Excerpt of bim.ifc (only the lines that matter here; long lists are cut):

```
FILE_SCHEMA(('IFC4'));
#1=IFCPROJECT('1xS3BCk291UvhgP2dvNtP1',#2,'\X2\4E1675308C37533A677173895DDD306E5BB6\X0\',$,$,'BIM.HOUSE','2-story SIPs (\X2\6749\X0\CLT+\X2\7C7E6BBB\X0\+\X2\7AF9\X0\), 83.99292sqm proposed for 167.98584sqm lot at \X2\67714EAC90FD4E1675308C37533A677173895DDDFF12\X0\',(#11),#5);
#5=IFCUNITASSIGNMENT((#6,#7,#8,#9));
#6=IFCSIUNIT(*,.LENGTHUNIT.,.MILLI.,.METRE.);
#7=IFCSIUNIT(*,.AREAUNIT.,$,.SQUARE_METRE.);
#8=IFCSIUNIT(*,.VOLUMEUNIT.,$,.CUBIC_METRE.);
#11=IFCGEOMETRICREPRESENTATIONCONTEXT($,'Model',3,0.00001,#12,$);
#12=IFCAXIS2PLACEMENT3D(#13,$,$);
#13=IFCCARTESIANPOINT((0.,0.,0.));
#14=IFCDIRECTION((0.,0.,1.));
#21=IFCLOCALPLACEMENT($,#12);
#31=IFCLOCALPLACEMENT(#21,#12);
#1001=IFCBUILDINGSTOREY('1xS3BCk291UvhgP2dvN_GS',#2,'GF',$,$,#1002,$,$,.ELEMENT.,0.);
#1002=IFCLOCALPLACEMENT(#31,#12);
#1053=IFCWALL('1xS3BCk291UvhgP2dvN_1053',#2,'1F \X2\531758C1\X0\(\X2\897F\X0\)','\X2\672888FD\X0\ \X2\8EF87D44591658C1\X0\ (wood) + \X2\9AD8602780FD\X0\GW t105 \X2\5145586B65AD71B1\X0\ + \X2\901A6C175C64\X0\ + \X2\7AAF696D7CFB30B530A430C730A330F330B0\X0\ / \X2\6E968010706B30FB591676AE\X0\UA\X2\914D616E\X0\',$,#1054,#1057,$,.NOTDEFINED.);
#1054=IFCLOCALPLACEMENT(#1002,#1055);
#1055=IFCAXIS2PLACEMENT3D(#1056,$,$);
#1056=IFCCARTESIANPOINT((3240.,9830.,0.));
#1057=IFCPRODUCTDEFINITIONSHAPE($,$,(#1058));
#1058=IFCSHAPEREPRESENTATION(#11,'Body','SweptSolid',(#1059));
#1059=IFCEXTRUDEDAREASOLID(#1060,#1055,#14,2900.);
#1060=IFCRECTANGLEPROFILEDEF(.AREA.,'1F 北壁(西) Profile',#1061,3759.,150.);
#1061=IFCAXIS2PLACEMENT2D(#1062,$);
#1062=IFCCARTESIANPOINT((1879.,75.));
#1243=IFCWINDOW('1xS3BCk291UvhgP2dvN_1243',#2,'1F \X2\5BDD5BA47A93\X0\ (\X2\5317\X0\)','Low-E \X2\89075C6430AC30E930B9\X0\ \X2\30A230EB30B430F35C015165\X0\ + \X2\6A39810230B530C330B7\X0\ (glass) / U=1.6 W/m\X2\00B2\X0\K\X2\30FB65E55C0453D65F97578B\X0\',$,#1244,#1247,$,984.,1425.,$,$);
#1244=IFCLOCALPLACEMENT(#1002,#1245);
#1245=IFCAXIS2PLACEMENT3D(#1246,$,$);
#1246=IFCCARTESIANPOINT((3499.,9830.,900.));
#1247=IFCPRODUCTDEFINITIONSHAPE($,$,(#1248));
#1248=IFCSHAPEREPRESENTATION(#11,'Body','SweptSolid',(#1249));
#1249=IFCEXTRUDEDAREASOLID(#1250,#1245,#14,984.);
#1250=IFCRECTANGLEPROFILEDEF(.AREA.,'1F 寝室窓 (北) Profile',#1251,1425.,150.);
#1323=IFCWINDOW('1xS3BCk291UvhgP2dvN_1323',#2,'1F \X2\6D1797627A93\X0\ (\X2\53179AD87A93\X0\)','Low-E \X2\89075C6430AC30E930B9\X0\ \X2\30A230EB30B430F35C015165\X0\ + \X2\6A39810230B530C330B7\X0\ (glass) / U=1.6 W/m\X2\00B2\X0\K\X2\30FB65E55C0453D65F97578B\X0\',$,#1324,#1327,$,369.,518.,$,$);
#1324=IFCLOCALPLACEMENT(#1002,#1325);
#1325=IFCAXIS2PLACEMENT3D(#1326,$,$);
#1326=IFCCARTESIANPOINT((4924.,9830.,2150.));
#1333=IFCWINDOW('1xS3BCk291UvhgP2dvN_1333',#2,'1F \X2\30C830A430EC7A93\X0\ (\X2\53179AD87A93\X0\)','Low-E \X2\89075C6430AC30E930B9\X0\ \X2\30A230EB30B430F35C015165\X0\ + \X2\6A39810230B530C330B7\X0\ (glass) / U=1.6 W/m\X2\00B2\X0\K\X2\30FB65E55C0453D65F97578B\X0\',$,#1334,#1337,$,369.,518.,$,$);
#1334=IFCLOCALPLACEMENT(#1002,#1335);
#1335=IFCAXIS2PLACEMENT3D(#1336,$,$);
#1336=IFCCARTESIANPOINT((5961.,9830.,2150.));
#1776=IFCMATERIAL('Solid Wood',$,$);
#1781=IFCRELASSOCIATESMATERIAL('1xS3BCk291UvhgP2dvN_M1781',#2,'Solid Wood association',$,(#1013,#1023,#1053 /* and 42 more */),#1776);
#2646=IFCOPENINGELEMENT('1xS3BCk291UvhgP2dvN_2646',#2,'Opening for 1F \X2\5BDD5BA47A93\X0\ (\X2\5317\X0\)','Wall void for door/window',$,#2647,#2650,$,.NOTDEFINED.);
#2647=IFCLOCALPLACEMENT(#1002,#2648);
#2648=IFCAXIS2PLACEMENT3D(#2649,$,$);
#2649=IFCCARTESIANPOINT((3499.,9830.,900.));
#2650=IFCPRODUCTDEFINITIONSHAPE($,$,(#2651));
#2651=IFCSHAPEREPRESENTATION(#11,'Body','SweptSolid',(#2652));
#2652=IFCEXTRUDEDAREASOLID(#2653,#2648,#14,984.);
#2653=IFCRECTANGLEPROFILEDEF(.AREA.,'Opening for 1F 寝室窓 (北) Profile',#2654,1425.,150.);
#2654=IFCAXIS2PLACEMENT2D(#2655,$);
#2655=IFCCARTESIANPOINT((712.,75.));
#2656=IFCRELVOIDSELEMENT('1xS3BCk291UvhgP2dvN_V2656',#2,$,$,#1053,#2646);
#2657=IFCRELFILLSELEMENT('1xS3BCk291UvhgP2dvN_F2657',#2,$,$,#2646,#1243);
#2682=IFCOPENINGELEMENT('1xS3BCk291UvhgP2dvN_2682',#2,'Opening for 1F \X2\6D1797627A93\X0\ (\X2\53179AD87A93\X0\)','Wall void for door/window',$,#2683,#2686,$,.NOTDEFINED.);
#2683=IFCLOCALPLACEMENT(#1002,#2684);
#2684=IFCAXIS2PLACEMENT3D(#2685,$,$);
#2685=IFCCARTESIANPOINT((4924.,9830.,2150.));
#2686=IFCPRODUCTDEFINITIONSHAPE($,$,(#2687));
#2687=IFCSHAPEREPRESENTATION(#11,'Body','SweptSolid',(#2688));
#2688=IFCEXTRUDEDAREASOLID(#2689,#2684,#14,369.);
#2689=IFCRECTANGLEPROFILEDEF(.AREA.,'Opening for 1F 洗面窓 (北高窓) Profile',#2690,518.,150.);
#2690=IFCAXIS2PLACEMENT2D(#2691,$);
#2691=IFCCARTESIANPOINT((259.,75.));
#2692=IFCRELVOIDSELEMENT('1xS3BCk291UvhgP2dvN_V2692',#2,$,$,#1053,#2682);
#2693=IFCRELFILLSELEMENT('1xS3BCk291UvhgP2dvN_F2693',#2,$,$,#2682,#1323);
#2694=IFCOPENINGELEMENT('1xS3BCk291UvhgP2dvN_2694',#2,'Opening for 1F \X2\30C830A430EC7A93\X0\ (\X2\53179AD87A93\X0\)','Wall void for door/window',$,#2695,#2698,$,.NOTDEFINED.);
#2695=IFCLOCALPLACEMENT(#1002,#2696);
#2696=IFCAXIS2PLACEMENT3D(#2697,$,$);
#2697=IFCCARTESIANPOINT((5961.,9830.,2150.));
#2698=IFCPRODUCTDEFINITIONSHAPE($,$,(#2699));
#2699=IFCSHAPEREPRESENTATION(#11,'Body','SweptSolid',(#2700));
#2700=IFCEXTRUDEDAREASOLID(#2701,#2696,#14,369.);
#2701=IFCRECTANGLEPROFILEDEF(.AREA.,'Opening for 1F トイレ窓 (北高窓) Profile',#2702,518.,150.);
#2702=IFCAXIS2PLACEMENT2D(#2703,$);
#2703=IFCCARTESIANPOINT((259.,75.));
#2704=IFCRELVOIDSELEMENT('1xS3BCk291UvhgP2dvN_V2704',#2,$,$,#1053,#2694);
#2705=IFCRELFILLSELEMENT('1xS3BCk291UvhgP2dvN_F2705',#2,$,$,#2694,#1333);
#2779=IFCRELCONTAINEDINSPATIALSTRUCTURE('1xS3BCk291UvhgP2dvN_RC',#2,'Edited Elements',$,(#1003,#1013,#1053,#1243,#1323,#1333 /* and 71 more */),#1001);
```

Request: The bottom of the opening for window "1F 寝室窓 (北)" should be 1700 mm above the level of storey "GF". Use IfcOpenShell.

```python
import numpy as np
import ifcopenshell
import ifcopenshell.api.geometry
import ifcopenshell.geom
import ifcopenshell.util.element
import ifcopenshell.util.placement
import ifcopenshell.util.shape
import ifcopenshell.util.unit

model = ifcopenshell.open("bim.ifc")
unit_scale = ifcopenshell.util.unit.calculate_unit_scale(model)

window = model.by_guid("1xS3BCk291UvhgP2dvN_1243")
opening = window.FillsVoids[0].RelatingOpeningElement
storey = ifcopenshell.util.element.get_container(window, ifc_class="IfcBuildingStorey")
level = ifcopenshell.util.placement.get_local_placement(storey.ObjectPlacement)[2, 3]

# The opening's origin need not be at the sill, so measure its lowest point.
shape = ifcopenshell.geom.create_shape(ifcopenshell.geom.settings(), opening)
bottom = ifcopenshell.util.shape.get_shape_bottom_elevation(shape, shape.geometry) / unit_scale
dz = level + 1.7 / unit_scale - bottom

shift = np.array([0.0, 0.0, dz])
# The window is not placed relative to its opening, so move both.
for product in (opening, window):
    matrix = ifcopenshell.util.placement.get_local_placement(product.ObjectPlacement)
    matrix[:3, 3] += shift
    ifcopenshell.api.geometry.edit_object_placement(model, product=product, matrix=matrix, is_si=False)

print(f"moved by {dz * unit_scale:+.3f} m")

model.write("bim_edited.ifc")
```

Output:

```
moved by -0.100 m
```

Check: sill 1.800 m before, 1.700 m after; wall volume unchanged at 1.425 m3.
